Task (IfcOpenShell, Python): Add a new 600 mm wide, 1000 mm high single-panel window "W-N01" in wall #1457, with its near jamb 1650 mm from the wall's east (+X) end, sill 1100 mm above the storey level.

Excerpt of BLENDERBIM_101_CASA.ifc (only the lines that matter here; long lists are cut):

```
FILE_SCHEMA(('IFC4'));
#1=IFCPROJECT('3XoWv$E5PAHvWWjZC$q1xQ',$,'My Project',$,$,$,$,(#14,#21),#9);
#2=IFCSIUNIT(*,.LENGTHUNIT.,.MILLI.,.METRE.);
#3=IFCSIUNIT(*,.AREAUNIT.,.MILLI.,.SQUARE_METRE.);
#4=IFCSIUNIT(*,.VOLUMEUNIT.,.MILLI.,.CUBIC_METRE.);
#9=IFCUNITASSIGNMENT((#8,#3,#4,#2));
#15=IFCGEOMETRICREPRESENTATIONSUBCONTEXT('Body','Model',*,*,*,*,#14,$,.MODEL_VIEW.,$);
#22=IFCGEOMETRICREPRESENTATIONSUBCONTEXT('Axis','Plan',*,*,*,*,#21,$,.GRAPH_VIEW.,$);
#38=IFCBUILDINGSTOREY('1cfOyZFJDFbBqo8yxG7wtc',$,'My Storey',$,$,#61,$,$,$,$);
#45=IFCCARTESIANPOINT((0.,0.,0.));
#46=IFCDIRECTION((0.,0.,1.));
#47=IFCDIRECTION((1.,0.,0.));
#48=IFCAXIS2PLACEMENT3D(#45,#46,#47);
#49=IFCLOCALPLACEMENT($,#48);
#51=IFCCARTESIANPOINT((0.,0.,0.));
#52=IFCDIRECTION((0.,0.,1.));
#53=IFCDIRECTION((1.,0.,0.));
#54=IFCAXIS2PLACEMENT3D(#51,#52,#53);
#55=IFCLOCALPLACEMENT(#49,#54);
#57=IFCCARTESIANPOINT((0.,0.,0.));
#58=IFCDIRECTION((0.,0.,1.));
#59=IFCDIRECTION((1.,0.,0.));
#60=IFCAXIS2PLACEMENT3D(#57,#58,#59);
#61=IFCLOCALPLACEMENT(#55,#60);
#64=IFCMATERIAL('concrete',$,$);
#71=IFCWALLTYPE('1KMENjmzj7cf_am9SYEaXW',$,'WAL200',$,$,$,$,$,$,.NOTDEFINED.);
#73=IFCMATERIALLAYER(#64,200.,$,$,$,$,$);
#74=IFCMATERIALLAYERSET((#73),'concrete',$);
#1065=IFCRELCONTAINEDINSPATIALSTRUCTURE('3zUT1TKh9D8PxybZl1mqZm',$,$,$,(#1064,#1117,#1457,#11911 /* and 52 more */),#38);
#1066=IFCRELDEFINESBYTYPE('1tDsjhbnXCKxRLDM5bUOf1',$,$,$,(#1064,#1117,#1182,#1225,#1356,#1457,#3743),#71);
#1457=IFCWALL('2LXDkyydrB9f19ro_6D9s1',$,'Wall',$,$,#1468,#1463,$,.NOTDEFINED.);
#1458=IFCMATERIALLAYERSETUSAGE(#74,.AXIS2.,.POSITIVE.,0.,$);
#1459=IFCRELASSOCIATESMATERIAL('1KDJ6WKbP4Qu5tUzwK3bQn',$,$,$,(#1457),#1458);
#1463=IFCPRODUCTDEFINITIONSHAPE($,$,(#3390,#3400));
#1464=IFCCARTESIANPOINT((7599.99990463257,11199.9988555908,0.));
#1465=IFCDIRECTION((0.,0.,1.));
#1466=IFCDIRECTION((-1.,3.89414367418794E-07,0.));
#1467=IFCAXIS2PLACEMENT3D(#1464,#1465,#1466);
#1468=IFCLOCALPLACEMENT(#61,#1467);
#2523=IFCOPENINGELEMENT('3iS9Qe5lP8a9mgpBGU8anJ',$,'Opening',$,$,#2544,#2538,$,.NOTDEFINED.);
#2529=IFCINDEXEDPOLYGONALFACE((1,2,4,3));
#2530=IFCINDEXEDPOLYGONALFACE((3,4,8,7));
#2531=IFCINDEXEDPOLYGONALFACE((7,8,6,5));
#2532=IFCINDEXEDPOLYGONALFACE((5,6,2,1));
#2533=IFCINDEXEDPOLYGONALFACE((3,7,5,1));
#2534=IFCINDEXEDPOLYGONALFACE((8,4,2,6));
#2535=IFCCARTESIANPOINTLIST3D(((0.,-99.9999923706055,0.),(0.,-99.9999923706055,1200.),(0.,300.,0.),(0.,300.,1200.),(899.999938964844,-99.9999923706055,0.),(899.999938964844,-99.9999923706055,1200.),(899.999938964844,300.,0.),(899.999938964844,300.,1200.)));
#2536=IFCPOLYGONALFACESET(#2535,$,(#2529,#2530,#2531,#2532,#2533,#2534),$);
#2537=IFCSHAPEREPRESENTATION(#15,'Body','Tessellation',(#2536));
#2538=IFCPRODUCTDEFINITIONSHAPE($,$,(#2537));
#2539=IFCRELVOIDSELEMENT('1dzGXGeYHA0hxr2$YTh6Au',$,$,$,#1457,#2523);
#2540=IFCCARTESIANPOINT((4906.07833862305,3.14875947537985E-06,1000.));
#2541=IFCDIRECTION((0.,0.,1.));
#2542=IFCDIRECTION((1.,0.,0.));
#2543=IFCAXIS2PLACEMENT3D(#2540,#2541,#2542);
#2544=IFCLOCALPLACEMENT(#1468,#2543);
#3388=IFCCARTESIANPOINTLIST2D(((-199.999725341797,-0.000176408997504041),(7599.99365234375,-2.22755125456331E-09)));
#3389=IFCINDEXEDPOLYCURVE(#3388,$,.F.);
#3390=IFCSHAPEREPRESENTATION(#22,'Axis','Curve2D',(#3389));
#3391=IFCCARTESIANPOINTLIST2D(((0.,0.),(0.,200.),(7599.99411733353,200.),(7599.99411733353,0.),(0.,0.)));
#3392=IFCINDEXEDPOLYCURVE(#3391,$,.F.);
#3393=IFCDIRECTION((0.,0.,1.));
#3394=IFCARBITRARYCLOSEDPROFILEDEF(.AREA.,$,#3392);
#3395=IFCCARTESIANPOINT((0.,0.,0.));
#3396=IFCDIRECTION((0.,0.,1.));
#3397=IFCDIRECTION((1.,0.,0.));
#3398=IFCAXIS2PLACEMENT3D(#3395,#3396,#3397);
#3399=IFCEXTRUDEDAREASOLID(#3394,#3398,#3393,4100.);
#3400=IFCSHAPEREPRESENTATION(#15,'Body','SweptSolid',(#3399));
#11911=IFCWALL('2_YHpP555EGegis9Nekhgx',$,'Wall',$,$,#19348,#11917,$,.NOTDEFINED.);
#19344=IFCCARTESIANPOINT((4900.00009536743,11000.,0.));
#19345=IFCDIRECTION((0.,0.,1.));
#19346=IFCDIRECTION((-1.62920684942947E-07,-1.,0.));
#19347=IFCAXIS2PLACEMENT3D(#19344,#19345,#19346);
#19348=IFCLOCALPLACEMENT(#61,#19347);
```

```python
import numpy as np
import ifcopenshell
import ifcopenshell.api.feature
import ifcopenshell.api.geometry
import ifcopenshell.api.root
import ifcopenshell.api.spatial
import ifcopenshell.geom
import ifcopenshell.util.element
import ifcopenshell.util.placement
import ifcopenshell.util.representation
import ifcopenshell.util.shape
import ifcopenshell.util.unit

model = ifcopenshell.open("BLENDERBIM_101_CASA.ifc")
unit_scale = ifcopenshell.util.unit.calculate_unit_scale(model)
settings = ifcopenshell.geom.settings()


def volume(element):
    """Net volume in cubic metres, openings subtracted."""
    shape = ifcopenshell.geom.create_shape(settings, element)
    return ifcopenshell.util.shape.get_volume(shape.geometry)


wall = model.by_id(1457)
storey = ifcopenshell.util.element.get_container(wall, ifc_class="IfcBuildingStorey")
context = ifcopenshell.util.representation.get_context(model, "Model", "Body", "MODEL_VIEW")
before = volume(wall)

width, height, from_end, sill = 0.6, 1, 1.65, 1.1  # metres

# The wall runs along its own X axis, and the end named is its -X end.
wall_shape = ifcopenshell.geom.create_shape(settings, wall)
x, y, z = ifcopenshell.util.shape.get_vertices(wall_shape.geometry).T
start = x.min() + from_end
face, thickness = float(y.min()), float(y.max() - y.min())
wall_matrix = ifcopenshell.util.placement.get_local_placement(wall.ObjectPlacement)
level = ifcopenshell.util.placement.get_local_placement(storey.ObjectPlacement)[2, 3]


def in_wall(x, y):
    """Placement at x, y metres in the wall's axes, at sill height."""
    matrix = wall_matrix.copy()
    matrix[:, 3] = wall_matrix @ np.array([x / unit_scale, y / unit_scale, 0.0, 1.0])
    matrix[2, 3] = level + sill / unit_scale
    return matrix


# Opening: a box that overshoots both wall faces by 50 mm.
opening = ifcopenshell.api.root.create_entity(model, ifc_class="IfcOpeningElement", predefined_type="OPENING")
box = ifcopenshell.api.geometry.add_wall_representation(
    model, context=context, length=width, height=height, thickness=thickness + 0.1
)
ifcopenshell.api.geometry.assign_representation(model, product=opening, representation=box)
ifcopenshell.api.geometry.edit_object_placement(model, product=opening, matrix=in_wall(start, face - 0.05), is_si=False)
ifcopenshell.api.feature.add_feature(model, feature=opening, element=wall)

window = ifcopenshell.api.root.create_entity(model, ifc_class="IfcWindow", name="W-N01", predefined_type="WINDOW")
window.OverallWidth, window.OverallHeight = width / unit_scale, height / unit_scale
window.PartitioningType = "SINGLE_PANEL"
body = ifcopenshell.api.geometry.add_window_representation(
    model,
    context=context,
    overall_width=window.OverallWidth,
    overall_height=window.OverallHeight,
    partition_type="SINGLE_PANEL",
)
ifcopenshell.api.geometry.assign_representation(model, product=window, representation=body)
ifcopenshell.api.spatial.assign_container(model, products=[window], relating_structure=storey)
ifcopenshell.api.feature.add_filling(model, opening=opening, element=window)

# Centre the window in the wall's thickness.
ifcopenshell.api.geometry.edit_object_placement(model, product=window, matrix=in_wall(start, face), is_si=False)
window_shape = ifcopenshell.geom.create_shape(settings, window)
depth = ifcopenshell.util.shape.get_vertices(window_shape.geometry)[:, 1]
offset = face + thickness / 2 - (depth.min() + depth.max()) / 2
ifcopenshell.api.geometry.edit_object_placement(model, product=window, matrix=in_wall(start, offset), is_si=False)

after = volume(wall)

print(f"wall volume {before:.3f} -> {after:.3f} m3")

model.write("BLENDERBIM_101_CASA_rev.ifc")
```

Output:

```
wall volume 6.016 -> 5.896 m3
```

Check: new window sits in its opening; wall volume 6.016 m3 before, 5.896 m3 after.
